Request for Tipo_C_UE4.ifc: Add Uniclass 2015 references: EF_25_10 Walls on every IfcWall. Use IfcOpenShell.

First a look at what the model holds.

```python
import ifcopenshell

model = ifcopenshell.open("Tipo_C_UE4.ifc")
print(model.schema)
print("classifications:", [c.Name for c in model.by_type("IfcClassification")])
for ifc_class in ("IfcDoor", "IfcRoof", "IfcStair", "IfcWall", "IfcWindow"):
    print(ifc_class, len(model.by_type(ifc_class)))
```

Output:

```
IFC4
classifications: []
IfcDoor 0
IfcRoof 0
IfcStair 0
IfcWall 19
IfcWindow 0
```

```python
import ifcopenshell
import ifcopenshell.api.classification

model = ifcopenshell.open("Tipo_C_UE4.ifc")

system = ifcopenshell.api.classification.add_classification(model, classification="Uniclass 2015")

codes = {
    "IfcWall": ("EF_25_10", "Walls"),
}
for ifc_class, (code, name) in codes.items():
    products = model.by_type(ifc_class)
    ifcopenshell.api.classification.add_reference(
        model, products=products, classification=system, identification=code, name=name
    )
    print(code, len(products))

model.write("Tipo_C_UE4-out.ifc")
```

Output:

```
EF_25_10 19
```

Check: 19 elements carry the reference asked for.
